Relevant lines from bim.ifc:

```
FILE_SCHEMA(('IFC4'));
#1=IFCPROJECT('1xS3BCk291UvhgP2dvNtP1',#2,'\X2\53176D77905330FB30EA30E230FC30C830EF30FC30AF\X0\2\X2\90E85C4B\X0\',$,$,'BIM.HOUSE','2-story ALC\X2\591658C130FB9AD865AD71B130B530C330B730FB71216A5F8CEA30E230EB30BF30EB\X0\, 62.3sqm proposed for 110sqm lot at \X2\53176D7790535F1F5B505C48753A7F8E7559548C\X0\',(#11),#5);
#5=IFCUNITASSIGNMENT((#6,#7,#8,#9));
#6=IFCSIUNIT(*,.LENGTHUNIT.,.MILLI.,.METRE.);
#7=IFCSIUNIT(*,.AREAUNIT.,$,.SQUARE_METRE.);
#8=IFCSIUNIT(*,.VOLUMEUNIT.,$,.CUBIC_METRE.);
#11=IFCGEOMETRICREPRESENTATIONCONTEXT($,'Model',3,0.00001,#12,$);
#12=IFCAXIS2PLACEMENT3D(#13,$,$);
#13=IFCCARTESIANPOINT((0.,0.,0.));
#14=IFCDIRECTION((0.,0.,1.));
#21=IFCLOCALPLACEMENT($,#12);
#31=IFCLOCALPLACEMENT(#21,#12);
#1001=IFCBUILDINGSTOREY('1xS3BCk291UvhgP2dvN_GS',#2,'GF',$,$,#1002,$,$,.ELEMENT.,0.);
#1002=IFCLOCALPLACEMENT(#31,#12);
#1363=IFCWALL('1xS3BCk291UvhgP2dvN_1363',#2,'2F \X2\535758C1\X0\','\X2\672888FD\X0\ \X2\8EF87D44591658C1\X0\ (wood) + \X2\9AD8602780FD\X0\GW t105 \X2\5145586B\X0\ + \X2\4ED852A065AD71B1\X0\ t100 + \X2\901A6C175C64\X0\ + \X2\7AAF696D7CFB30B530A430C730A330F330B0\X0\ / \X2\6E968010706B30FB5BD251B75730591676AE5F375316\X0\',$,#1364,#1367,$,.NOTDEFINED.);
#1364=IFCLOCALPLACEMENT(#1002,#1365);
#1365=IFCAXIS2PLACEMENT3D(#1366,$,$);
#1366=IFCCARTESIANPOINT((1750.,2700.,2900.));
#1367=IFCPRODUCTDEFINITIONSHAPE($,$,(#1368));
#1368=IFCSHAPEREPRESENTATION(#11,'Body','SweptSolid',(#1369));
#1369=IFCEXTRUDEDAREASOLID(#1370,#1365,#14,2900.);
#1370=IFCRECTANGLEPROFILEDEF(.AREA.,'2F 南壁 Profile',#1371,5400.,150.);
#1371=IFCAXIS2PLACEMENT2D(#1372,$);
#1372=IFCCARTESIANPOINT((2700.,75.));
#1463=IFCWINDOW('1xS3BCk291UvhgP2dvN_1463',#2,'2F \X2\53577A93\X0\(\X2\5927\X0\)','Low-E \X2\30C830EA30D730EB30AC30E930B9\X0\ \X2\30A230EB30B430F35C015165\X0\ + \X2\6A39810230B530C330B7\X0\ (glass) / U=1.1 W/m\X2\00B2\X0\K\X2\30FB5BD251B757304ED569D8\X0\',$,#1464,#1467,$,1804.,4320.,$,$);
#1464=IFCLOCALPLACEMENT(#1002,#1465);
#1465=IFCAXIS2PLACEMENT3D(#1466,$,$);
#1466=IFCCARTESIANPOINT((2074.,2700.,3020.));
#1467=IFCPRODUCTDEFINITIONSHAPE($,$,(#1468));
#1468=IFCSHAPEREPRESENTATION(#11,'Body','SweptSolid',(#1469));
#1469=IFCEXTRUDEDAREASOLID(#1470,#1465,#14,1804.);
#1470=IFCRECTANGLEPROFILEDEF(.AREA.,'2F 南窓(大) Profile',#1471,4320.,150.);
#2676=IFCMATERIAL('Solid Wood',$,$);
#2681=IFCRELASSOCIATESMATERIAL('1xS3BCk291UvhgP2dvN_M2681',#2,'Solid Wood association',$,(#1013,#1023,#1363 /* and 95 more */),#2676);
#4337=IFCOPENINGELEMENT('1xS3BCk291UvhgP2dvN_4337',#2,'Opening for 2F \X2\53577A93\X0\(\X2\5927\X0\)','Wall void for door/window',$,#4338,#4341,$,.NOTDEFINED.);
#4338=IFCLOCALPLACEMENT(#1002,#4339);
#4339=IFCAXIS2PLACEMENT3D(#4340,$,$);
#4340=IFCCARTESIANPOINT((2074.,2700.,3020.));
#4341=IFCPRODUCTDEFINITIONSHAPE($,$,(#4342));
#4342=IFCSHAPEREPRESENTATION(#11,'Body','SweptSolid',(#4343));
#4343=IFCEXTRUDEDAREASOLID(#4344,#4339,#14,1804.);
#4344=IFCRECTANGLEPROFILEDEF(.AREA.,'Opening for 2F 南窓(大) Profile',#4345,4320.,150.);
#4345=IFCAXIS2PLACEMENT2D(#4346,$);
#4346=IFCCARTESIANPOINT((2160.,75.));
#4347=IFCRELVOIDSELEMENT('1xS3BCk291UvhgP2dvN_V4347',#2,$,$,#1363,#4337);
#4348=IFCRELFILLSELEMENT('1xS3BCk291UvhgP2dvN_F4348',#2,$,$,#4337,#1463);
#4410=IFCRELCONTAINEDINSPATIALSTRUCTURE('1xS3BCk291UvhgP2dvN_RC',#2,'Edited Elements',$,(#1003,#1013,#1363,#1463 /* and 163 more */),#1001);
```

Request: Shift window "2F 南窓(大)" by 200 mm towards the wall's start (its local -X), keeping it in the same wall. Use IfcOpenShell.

```python
import ifcopenshell
import ifcopenshell.api.geometry
import ifcopenshell.util.placement
import ifcopenshell.util.unit

model = ifcopenshell.open("bim.ifc")
unit_scale = ifcopenshell.util.unit.calculate_unit_scale(model)

window = model.by_guid("1xS3BCk291UvhgP2dvN_1463")
opening = window.FillsVoids[0].RelatingOpeningElement
wall = opening.VoidsElements[0].RelatingBuildingElement

wall_matrix = ifcopenshell.util.placement.get_local_placement(wall.ObjectPlacement)
shift = wall_matrix[:3, 0] * -0.2 / unit_scale
before = ifcopenshell.util.placement.get_local_placement(window.ObjectPlacement)[:3, 3].copy()

# The window is not placed relative to its opening, so move both.
for product in (opening, window):
    matrix = ifcopenshell.util.placement.get_local_placement(product.ObjectPlacement)
    matrix[:3, 3] += shift
    ifcopenshell.api.geometry.edit_object_placement(model, product=product, matrix=matrix, is_si=False)

after = ifcopenshell.util.placement.get_local_placement(window.ObjectPlacement)[:3, 3]
print("window moved by", (after - before).round(3) + 0.0)

model.write("bim_rev.ifc")
```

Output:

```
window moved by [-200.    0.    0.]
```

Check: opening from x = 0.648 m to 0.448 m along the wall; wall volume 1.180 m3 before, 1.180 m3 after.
